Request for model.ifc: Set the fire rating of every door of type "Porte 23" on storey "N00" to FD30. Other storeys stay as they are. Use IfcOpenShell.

First a look at what the model holds.

```python
import ifcopenshell
import ifcopenshell.util.element

model = ifcopenshell.open("model.ifc")
print(model.schema)
storey = next(s for s in model.by_type("IfcBuildingStorey") if s.Name == "N00")
doors = [e for e in ifcopenshell.util.element.get_decomposition(storey) if e.is_a("IfcDoor")]
seen = {}
for e in doors:
    element_type = ifcopenshell.util.element.get_type(e)
    key = (element_type.Name if element_type != e and element_type else None, ifcopenshell.util.element.get_pset(e, "Pset_DoorCommon", "FireRating"))
    seen[key] = seen.get(key, 0) + 1
for (name, value), count in sorted(seen.items(), key=str):
    print(count, "x", name, "|", value)
```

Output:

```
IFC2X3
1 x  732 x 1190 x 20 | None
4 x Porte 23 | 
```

```python
import ifcopenshell
import ifcopenshell.api.pset
import ifcopenshell.util.element

model = ifcopenshell.open("model.ifc")

storey = next(s for s in model.by_type("IfcBuildingStorey") if s.Name == "N00")
doors = [e for e in ifcopenshell.util.element.get_decomposition(storey) if e.is_a("IfcDoor")]

count = 0
for e in doors:
    element_type = ifcopenshell.util.element.get_type(e)
    if element_type in (None, e) or element_type.Name != "Porte 23":
        continue
    # add_pset returns the element's existing set when there is one.
    pset = ifcopenshell.api.pset.add_pset(model, product=e, name="Pset_DoorCommon")
    ifcopenshell.api.pset.edit_pset(model, pset=pset, properties={"FireRating": "FD30"})
    count += 1

print(count, "doors updated")

model.write("model_updated.ifc")
```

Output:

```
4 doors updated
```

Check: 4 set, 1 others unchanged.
